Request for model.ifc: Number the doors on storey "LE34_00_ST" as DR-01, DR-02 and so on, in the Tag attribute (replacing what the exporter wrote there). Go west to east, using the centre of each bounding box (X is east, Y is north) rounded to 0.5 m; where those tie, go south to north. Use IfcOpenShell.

First a look at what the model holds.

```python
import ifcopenshell
import ifcopenshell.util.element
import ifcopenshell.util.placement

model = ifcopenshell.open("model.ifc")
print(model.schema)
storey = next(s for s in model.by_type("IfcBuildingStorey") if s.Name == "LE34_00_ST")
doors = [e for e in ifcopenshell.util.element.get_decomposition(storey) if e.is_a("IfcDoor")]
for e in sorted(doors, key=lambda e: e.id()):
    origin = ifcopenshell.util.placement.get_local_placement(e.ObjectPlacement)[:3, 3]
    print(e.id(), e.Tag, e.Name, origin.round(2) + 0.0, sep=" | ")
```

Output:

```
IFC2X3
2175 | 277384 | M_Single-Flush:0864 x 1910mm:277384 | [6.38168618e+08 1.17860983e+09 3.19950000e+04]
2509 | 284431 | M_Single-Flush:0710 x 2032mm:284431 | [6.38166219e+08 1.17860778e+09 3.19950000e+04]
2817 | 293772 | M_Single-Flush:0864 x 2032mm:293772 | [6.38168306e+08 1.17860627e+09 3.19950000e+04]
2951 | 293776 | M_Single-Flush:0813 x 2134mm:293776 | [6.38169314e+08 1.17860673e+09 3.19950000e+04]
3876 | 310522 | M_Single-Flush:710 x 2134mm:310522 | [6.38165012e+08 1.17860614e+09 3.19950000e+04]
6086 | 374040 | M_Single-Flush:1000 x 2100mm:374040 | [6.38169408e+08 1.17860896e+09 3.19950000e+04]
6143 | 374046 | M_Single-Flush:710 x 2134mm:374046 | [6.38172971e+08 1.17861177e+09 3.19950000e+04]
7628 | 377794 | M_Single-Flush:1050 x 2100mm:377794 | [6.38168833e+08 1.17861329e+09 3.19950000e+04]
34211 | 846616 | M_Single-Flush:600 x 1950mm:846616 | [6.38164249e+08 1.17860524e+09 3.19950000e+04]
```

```python
import ifcopenshell
import ifcopenshell.geom
import ifcopenshell.util.element
import ifcopenshell.util.shape

model = ifcopenshell.open("model.ifc")
settings = ifcopenshell.geom.settings()
settings.set("use-world-coords", True)


def centre(element):
    shape = ifcopenshell.geom.create_shape(settings, element)
    return ifcopenshell.util.shape.get_bbox_centroid(shape.geometry)


storey = next(s for s in model.by_type("IfcBuildingStorey") if s.Name == "LE34_00_ST")
doors = [e for e in ifcopenshell.util.element.get_decomposition(storey) if e.is_a("IfcDoor")]

# Insertion points can sit at a corner or the storey origin, so sort by the geometry (in metres).
centres = {e: centre(e) for e in doors}
doors.sort(key=lambda e: (round(centres[e][0] / 0.5), centres[e][1]))

for i, e in enumerate(doors, start=1):
    number = f"DR-{i:02d}"
    e.Tag = number
    print(e.id(), number)

model.write("model-out.ifc")
```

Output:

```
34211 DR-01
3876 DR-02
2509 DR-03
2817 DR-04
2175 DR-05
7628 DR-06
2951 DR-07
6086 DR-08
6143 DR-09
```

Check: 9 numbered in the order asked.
